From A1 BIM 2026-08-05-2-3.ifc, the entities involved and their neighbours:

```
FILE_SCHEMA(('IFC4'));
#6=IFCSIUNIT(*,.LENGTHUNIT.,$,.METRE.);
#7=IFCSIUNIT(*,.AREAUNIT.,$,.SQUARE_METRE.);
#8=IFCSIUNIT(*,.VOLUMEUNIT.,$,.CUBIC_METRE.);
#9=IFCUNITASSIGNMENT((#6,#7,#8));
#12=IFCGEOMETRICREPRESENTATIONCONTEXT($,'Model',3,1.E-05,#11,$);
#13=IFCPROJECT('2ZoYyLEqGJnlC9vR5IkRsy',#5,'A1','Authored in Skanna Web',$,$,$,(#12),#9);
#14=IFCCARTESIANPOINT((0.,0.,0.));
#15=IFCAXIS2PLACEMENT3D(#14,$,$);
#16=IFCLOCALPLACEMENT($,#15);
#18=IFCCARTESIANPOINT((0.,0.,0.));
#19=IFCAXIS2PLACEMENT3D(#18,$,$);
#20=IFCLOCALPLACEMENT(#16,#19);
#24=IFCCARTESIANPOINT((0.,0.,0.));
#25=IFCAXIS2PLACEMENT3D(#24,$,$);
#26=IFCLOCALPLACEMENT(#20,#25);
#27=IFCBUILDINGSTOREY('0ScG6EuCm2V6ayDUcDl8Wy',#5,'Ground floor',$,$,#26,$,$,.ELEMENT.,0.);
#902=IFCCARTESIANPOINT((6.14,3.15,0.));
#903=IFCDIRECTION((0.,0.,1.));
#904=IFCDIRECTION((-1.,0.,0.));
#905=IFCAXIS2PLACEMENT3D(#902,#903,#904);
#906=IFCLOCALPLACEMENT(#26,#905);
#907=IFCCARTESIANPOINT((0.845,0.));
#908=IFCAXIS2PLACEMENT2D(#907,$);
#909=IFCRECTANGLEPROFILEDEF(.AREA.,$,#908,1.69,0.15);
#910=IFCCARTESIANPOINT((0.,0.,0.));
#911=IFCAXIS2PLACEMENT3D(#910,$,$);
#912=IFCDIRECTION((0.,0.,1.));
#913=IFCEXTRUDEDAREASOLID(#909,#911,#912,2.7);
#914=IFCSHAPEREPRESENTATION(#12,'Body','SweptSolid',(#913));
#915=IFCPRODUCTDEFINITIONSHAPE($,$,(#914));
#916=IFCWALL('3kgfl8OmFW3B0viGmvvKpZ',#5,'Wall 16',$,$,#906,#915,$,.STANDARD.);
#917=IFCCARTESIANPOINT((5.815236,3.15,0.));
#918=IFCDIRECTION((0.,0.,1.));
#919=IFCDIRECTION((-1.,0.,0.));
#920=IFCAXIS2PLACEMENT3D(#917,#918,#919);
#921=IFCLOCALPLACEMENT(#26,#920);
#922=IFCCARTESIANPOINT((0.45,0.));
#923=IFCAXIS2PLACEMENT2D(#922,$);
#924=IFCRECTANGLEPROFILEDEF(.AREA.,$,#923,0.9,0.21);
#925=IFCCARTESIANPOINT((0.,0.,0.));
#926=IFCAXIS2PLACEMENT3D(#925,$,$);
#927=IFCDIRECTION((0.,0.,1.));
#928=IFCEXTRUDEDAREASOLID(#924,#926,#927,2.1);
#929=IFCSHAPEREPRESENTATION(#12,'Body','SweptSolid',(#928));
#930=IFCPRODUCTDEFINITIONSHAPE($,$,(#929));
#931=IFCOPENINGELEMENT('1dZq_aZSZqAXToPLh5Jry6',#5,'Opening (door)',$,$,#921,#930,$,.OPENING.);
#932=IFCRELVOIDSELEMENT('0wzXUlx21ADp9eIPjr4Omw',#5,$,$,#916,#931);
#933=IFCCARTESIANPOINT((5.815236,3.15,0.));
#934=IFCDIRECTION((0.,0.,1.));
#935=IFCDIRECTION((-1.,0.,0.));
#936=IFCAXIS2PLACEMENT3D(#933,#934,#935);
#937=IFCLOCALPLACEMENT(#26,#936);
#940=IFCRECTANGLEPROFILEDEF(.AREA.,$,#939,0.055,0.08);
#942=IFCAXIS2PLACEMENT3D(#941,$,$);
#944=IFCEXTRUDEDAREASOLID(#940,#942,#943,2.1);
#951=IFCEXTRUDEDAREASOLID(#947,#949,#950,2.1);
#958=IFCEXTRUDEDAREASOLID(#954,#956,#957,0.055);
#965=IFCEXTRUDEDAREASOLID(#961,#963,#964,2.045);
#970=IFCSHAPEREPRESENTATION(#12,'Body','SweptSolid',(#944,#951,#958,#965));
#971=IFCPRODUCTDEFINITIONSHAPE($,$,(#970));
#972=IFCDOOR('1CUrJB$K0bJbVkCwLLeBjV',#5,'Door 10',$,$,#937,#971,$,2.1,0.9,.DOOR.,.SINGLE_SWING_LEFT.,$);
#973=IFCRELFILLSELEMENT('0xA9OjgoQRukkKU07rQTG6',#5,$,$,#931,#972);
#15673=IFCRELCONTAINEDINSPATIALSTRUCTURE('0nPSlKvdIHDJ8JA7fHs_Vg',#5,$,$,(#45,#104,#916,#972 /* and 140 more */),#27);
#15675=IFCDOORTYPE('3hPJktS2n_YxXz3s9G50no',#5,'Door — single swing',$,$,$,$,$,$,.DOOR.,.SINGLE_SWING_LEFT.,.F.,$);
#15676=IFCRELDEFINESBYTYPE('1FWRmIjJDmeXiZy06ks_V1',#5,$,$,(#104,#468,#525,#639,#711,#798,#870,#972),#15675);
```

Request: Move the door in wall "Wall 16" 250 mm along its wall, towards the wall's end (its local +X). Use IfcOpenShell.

```python
import ifcopenshell
import ifcopenshell.api.geometry
import ifcopenshell.util.placement
import ifcopenshell.util.unit

model = ifcopenshell.open("A1 BIM 2026-08-05-2-3.ifc")
unit_scale = ifcopenshell.util.unit.calculate_unit_scale(model)

door = model.by_id(972)
opening = door.FillsVoids[0].RelatingOpeningElement
wall = opening.VoidsElements[0].RelatingBuildingElement

wall_matrix = ifcopenshell.util.placement.get_local_placement(wall.ObjectPlacement)
shift = wall_matrix[:3, 0] * 0.25 / unit_scale
before = ifcopenshell.util.placement.get_local_placement(door.ObjectPlacement)[:3, 3].copy()

# The door is not placed relative to its opening, so move both.
for product in (opening, door):
    matrix = ifcopenshell.util.placement.get_local_placement(product.ObjectPlacement)
    matrix[:3, 3] += shift
    ifcopenshell.api.geometry.edit_object_placement(model, product=product, matrix=matrix, is_si=False)

after = ifcopenshell.util.placement.get_local_placement(door.ObjectPlacement)[:3, 3]
print("door moved by", (after - before).round(3) + 0.0)

model.write("A1 BIM 2026-08-05-2-3_edited.ifc")
```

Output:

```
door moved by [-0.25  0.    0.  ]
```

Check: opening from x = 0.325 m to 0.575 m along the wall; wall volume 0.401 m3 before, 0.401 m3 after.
